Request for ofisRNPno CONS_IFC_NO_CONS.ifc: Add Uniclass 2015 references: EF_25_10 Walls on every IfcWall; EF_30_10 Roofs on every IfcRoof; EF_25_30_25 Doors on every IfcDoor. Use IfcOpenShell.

First a look at what the model holds.

```python
import ifcopenshell

model = ifcopenshell.open("ofisRNPno CONS_IFC_NO_CONS.ifc")
print(model.schema)
print("classifications:", [c.Name for c in model.by_type("IfcClassification")])
for ifc_class in ("IfcDoor", "IfcRoof", "IfcStair", "IfcWall", "IfcWindow"):
    print(ifc_class, len(model.by_type(ifc_class)))
```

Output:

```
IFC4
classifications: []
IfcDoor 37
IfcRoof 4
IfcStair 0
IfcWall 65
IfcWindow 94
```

```python
import ifcopenshell
import ifcopenshell.api.classification

model = ifcopenshell.open("ofisRNPno CONS_IFC_NO_CONS.ifc")

system = ifcopenshell.api.classification.add_classification(model, classification="Uniclass 2015")

codes = {
    "IfcWall": ("EF_25_10", "Walls"),
    "IfcRoof": ("EF_30_10", "Roofs"),
    "IfcDoor": ("EF_25_30_25", "Doors"),
}
for ifc_class, (code, name) in codes.items():
    products = model.by_type(ifc_class)
    ifcopenshell.api.classification.add_reference(
        model, products=products, classification=system, identification=code, name=name
    )
    print(code, len(products))

model.write("ofisRNPno CONS_IFC_NO_CONS_updated.ifc")
```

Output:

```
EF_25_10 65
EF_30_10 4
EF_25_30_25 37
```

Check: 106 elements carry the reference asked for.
